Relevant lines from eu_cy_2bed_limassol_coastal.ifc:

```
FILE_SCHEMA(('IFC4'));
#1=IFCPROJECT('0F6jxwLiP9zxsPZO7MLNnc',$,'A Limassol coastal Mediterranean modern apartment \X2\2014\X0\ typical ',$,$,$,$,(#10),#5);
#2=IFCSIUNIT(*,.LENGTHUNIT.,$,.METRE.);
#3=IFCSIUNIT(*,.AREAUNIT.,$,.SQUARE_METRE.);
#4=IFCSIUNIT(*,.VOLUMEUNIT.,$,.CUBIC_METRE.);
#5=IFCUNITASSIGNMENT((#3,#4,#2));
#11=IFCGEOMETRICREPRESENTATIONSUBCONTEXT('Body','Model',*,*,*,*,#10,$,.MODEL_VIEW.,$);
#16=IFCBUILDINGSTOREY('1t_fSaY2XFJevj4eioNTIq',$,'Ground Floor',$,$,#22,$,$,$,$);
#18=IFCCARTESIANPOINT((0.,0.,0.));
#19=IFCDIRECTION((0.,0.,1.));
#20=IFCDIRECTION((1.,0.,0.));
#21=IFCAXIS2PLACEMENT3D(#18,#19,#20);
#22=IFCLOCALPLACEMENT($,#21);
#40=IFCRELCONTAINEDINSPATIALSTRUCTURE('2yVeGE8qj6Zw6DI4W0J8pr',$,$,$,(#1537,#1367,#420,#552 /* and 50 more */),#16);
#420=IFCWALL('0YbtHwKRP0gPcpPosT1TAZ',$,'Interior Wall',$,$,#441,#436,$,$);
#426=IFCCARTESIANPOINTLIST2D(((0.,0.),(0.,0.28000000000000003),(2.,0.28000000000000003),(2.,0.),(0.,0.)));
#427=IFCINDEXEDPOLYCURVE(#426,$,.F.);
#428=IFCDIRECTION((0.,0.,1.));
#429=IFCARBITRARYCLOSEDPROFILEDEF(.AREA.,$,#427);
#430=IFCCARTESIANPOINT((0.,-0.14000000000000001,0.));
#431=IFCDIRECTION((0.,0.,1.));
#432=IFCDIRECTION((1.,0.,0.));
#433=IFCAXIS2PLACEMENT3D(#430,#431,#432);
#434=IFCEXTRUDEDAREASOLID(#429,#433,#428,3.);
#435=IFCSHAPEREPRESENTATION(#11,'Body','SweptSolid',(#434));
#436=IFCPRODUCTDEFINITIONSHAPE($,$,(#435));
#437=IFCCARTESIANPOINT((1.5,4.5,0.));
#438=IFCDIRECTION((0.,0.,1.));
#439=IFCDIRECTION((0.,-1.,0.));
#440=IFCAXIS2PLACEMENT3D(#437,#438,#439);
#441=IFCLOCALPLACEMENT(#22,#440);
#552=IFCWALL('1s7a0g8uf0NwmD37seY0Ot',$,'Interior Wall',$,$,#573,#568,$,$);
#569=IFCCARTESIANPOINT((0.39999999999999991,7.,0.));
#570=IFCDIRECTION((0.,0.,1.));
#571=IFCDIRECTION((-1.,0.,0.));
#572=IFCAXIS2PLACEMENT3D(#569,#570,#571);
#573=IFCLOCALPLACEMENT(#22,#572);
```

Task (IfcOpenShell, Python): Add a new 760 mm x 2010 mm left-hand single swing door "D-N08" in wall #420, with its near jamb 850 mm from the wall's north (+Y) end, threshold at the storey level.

```python
import numpy as np
import ifcopenshell
import ifcopenshell.api.feature
import ifcopenshell.api.geometry
import ifcopenshell.api.root
import ifcopenshell.api.spatial
import ifcopenshell.geom
import ifcopenshell.util.element
import ifcopenshell.util.placement
import ifcopenshell.util.representation
import ifcopenshell.util.shape
import ifcopenshell.util.unit

model = ifcopenshell.open("eu_cy_2bed_limassol_coastal.ifc")
unit_scale = ifcopenshell.util.unit.calculate_unit_scale(model)
settings = ifcopenshell.geom.settings()


def volume(element):
    """Net volume in cubic metres, openings subtracted."""
    shape = ifcopenshell.geom.create_shape(settings, element)
    return ifcopenshell.util.shape.get_volume(shape.geometry)


wall = model.by_guid("0YbtHwKRP0gPcpPosT1TAZ")
storey = ifcopenshell.util.element.get_container(wall, ifc_class="IfcBuildingStorey")
context = ifcopenshell.util.representation.get_context(model, "Model", "Body", "MODEL_VIEW")
before = volume(wall)

width, height, from_end, sill = 0.76, 2.01, 0.85, 0.0  # metres

# The wall runs along its own X axis, and the end named is its -X end.
wall_shape = ifcopenshell.geom.create_shape(settings, wall)
x, y, z = ifcopenshell.util.shape.get_vertices(wall_shape.geometry).T
start = x.min() + from_end
face, thickness = float(y.min()), float(y.max() - y.min())
wall_matrix = ifcopenshell.util.placement.get_local_placement(wall.ObjectPlacement)
level = ifcopenshell.util.placement.get_local_placement(storey.ObjectPlacement)[2, 3]


def in_wall(x, y):
    """Placement at x, y metres in the wall's axes, at sill height."""
    matrix = wall_matrix.copy()
    matrix[:, 3] = wall_matrix @ np.array([x / unit_scale, y / unit_scale, 0.0, 1.0])
    matrix[2, 3] = level + sill / unit_scale
    return matrix


# Opening: a box that overshoots both wall faces by 50 mm.
opening = ifcopenshell.api.root.create_entity(model, ifc_class="IfcOpeningElement", predefined_type="OPENING")
box = ifcopenshell.api.geometry.add_wall_representation(
    model, context=context, length=width, height=height, thickness=thickness + 0.1
)
ifcopenshell.api.geometry.assign_representation(model, product=opening, representation=box)
ifcopenshell.api.geometry.edit_object_placement(model, product=opening, matrix=in_wall(start, face - 0.05), is_si=False)
ifcopenshell.api.feature.add_feature(model, feature=opening, element=wall)

door = ifcopenshell.api.root.create_entity(model, ifc_class="IfcDoor", name="D-N08", predefined_type="DOOR")
door.OverallWidth, door.OverallHeight = width / unit_scale, height / unit_scale
door.OperationType = "SINGLE_SWING_LEFT"
body = ifcopenshell.api.geometry.add_door_representation(
    model,
    context=context,
    overall_width=door.OverallWidth,
    overall_height=door.OverallHeight,
    operation_type="SINGLE_SWING_LEFT",
    lining_properties={"LiningDepth": thickness / unit_scale, "ThresholdDepth": thickness / unit_scale},
)
ifcopenshell.api.geometry.assign_representation(model, product=door, representation=body)
ifcopenshell.api.spatial.assign_container(model, products=[door], relating_structure=storey)
ifcopenshell.api.feature.add_filling(model, opening=opening, element=door)

# The lining spans the wall, so the door starts at the wall face.
ifcopenshell.api.geometry.edit_object_placement(model, product=door, matrix=in_wall(start, face), is_si=False)

after = volume(wall)

print(f"wall volume {before:.3f} -> {after:.3f} m3")

model.write("eu_cy_2bed_limassol_coastal_edited.ifc")
```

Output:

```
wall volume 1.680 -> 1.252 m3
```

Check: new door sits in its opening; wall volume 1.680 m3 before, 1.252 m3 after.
